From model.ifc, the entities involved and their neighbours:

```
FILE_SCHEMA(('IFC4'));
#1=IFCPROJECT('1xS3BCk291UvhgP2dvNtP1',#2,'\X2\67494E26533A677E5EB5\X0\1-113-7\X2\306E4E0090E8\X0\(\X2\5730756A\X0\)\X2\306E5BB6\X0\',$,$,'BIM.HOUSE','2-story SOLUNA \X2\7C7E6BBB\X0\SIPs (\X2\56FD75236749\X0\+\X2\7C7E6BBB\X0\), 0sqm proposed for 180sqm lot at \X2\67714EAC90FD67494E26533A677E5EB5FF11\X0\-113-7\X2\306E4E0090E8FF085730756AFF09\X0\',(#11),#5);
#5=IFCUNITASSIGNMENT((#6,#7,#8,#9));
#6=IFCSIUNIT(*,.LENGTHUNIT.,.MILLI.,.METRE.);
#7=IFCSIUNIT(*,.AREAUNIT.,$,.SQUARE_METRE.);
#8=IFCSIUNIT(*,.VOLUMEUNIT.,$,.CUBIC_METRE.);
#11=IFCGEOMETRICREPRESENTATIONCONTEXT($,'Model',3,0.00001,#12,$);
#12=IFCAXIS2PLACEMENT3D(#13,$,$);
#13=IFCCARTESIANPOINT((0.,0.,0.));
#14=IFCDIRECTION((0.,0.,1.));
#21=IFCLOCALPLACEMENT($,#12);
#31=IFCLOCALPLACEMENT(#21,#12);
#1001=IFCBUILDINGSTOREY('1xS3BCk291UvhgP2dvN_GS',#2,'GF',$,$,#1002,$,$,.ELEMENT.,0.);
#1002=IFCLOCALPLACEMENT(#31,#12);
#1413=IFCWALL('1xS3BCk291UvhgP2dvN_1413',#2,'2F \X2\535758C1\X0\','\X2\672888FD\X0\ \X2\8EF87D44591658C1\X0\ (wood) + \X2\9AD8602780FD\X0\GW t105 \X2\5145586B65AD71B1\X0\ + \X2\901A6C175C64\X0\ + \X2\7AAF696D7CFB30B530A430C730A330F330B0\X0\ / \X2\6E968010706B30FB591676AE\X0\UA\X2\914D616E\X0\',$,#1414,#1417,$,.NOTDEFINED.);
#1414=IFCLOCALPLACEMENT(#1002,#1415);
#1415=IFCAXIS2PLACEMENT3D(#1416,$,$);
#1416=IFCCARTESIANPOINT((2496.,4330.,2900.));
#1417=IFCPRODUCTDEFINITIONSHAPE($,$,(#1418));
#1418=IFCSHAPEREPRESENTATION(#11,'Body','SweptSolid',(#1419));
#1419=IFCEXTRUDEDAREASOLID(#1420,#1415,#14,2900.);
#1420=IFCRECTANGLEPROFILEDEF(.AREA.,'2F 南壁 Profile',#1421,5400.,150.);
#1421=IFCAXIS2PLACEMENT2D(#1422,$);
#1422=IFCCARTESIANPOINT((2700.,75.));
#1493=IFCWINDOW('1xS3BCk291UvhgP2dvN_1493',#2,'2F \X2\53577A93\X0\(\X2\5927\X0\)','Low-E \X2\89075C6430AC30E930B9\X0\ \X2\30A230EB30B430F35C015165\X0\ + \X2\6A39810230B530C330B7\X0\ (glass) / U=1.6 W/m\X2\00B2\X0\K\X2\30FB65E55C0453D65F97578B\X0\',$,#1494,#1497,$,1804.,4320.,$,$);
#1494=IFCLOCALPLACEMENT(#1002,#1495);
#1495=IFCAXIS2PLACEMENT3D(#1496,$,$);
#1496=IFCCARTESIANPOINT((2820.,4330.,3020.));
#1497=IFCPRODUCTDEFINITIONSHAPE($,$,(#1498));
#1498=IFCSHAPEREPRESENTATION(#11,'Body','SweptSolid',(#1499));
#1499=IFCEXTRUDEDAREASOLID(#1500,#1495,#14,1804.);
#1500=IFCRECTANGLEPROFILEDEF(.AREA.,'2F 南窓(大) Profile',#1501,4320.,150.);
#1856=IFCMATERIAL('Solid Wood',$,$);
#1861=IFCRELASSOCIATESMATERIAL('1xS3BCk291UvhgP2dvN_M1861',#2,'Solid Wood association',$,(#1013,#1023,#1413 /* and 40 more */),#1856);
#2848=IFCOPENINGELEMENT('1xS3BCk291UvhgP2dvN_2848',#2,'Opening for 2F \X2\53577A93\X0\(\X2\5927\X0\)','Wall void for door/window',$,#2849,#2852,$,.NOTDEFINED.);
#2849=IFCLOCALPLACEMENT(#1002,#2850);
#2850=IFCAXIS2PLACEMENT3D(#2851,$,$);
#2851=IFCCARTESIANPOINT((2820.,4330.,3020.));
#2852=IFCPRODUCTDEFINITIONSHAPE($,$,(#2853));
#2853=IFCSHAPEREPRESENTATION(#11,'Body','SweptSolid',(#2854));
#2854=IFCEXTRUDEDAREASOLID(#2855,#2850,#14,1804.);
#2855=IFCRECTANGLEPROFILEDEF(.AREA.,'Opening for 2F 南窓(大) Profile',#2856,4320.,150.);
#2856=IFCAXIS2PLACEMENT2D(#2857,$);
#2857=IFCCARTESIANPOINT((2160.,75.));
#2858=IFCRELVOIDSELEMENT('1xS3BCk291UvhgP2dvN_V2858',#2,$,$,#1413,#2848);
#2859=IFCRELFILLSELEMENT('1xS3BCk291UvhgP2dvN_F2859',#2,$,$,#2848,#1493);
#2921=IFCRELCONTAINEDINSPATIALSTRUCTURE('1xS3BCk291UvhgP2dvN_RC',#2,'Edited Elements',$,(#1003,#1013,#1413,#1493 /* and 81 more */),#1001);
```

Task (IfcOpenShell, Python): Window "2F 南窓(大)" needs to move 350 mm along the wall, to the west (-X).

```python
import ifcopenshell
import ifcopenshell.api.geometry
import ifcopenshell.util.placement

model = ifcopenshell.open("model.ifc")

window = model.by_id(1493)
opening = window.FillsVoids[0].RelatingOpeningElement
wall = opening.VoidsElements[0].RelatingBuildingElement

wall_matrix = ifcopenshell.util.placement.get_local_placement(wall.ObjectPlacement)
shift = wall_matrix[:3, 0] * -350.0
before = ifcopenshell.util.placement.get_local_placement(window.ObjectPlacement)[:3, 3].copy()

# The window is not placed relative to its opening, so move both.
for product in (opening, window):
    matrix = ifcopenshell.util.placement.get_local_placement(product.ObjectPlacement)
    matrix[:3, 3] += shift
    ifcopenshell.api.geometry.edit_object_placement(model, product=product, matrix=matrix, is_si=False)

after = ifcopenshell.util.placement.get_local_placement(window.ObjectPlacement)[:3, 3]
print("window moved by", (after - before).round(3) + 0.0)

model.write("model_rev.ifc")
```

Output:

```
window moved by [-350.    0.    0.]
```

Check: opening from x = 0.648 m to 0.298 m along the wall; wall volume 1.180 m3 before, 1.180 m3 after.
